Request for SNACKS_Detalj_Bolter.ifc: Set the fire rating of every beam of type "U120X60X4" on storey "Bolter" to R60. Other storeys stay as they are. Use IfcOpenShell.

First a look at what the model holds.

```python
import ifcopenshell
import ifcopenshell.util.element

model = ifcopenshell.open("SNACKS_Detalj_Bolter.ifc")
print(model.schema)
storey = next(s for s in model.by_type("IfcBuildingStorey") if s.Name == "Bolter")
beams = [e for e in ifcopenshell.util.element.get_decomposition(storey) if e.is_a("IfcBeam")]
seen = {}
for e in beams:
    element_type = ifcopenshell.util.element.get_type(e)
    key = (element_type.Name if element_type != e and element_type else None, ifcopenshell.util.element.get_pset(e, "Pset_BeamCommon", "FireRating"))
    seen[key] = seen.get(key, 0) + 1
for (name, value), count in sorted(seen.items(), key=str):
    print(count, "x", name, "|", value)
```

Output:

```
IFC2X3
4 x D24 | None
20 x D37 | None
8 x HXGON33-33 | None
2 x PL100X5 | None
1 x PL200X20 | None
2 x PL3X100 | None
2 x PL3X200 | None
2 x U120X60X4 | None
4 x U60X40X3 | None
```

```python
import ifcopenshell
import ifcopenshell.api.pset
import ifcopenshell.util.element

model = ifcopenshell.open("SNACKS_Detalj_Bolter.ifc")

storey = next(s for s in model.by_type("IfcBuildingStorey") if s.Name == "Bolter")
beams = [e for e in ifcopenshell.util.element.get_decomposition(storey) if e.is_a("IfcBeam")]

count = 0
for e in beams:
    element_type = ifcopenshell.util.element.get_type(e)
    if element_type in (None, e) or element_type.Name != "U120X60X4":
        continue
    # add_pset returns the element's existing set when there is one.
    pset = ifcopenshell.api.pset.add_pset(model, product=e, name="Pset_BeamCommon")
    ifcopenshell.api.pset.edit_pset(model, pset=pset, properties={"FireRating": "R60"})
    count += 1

print(count, "beams updated")

model.write("SNACKS_Detalj_Bolter_edited.ifc")
```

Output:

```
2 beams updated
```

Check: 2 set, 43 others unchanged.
